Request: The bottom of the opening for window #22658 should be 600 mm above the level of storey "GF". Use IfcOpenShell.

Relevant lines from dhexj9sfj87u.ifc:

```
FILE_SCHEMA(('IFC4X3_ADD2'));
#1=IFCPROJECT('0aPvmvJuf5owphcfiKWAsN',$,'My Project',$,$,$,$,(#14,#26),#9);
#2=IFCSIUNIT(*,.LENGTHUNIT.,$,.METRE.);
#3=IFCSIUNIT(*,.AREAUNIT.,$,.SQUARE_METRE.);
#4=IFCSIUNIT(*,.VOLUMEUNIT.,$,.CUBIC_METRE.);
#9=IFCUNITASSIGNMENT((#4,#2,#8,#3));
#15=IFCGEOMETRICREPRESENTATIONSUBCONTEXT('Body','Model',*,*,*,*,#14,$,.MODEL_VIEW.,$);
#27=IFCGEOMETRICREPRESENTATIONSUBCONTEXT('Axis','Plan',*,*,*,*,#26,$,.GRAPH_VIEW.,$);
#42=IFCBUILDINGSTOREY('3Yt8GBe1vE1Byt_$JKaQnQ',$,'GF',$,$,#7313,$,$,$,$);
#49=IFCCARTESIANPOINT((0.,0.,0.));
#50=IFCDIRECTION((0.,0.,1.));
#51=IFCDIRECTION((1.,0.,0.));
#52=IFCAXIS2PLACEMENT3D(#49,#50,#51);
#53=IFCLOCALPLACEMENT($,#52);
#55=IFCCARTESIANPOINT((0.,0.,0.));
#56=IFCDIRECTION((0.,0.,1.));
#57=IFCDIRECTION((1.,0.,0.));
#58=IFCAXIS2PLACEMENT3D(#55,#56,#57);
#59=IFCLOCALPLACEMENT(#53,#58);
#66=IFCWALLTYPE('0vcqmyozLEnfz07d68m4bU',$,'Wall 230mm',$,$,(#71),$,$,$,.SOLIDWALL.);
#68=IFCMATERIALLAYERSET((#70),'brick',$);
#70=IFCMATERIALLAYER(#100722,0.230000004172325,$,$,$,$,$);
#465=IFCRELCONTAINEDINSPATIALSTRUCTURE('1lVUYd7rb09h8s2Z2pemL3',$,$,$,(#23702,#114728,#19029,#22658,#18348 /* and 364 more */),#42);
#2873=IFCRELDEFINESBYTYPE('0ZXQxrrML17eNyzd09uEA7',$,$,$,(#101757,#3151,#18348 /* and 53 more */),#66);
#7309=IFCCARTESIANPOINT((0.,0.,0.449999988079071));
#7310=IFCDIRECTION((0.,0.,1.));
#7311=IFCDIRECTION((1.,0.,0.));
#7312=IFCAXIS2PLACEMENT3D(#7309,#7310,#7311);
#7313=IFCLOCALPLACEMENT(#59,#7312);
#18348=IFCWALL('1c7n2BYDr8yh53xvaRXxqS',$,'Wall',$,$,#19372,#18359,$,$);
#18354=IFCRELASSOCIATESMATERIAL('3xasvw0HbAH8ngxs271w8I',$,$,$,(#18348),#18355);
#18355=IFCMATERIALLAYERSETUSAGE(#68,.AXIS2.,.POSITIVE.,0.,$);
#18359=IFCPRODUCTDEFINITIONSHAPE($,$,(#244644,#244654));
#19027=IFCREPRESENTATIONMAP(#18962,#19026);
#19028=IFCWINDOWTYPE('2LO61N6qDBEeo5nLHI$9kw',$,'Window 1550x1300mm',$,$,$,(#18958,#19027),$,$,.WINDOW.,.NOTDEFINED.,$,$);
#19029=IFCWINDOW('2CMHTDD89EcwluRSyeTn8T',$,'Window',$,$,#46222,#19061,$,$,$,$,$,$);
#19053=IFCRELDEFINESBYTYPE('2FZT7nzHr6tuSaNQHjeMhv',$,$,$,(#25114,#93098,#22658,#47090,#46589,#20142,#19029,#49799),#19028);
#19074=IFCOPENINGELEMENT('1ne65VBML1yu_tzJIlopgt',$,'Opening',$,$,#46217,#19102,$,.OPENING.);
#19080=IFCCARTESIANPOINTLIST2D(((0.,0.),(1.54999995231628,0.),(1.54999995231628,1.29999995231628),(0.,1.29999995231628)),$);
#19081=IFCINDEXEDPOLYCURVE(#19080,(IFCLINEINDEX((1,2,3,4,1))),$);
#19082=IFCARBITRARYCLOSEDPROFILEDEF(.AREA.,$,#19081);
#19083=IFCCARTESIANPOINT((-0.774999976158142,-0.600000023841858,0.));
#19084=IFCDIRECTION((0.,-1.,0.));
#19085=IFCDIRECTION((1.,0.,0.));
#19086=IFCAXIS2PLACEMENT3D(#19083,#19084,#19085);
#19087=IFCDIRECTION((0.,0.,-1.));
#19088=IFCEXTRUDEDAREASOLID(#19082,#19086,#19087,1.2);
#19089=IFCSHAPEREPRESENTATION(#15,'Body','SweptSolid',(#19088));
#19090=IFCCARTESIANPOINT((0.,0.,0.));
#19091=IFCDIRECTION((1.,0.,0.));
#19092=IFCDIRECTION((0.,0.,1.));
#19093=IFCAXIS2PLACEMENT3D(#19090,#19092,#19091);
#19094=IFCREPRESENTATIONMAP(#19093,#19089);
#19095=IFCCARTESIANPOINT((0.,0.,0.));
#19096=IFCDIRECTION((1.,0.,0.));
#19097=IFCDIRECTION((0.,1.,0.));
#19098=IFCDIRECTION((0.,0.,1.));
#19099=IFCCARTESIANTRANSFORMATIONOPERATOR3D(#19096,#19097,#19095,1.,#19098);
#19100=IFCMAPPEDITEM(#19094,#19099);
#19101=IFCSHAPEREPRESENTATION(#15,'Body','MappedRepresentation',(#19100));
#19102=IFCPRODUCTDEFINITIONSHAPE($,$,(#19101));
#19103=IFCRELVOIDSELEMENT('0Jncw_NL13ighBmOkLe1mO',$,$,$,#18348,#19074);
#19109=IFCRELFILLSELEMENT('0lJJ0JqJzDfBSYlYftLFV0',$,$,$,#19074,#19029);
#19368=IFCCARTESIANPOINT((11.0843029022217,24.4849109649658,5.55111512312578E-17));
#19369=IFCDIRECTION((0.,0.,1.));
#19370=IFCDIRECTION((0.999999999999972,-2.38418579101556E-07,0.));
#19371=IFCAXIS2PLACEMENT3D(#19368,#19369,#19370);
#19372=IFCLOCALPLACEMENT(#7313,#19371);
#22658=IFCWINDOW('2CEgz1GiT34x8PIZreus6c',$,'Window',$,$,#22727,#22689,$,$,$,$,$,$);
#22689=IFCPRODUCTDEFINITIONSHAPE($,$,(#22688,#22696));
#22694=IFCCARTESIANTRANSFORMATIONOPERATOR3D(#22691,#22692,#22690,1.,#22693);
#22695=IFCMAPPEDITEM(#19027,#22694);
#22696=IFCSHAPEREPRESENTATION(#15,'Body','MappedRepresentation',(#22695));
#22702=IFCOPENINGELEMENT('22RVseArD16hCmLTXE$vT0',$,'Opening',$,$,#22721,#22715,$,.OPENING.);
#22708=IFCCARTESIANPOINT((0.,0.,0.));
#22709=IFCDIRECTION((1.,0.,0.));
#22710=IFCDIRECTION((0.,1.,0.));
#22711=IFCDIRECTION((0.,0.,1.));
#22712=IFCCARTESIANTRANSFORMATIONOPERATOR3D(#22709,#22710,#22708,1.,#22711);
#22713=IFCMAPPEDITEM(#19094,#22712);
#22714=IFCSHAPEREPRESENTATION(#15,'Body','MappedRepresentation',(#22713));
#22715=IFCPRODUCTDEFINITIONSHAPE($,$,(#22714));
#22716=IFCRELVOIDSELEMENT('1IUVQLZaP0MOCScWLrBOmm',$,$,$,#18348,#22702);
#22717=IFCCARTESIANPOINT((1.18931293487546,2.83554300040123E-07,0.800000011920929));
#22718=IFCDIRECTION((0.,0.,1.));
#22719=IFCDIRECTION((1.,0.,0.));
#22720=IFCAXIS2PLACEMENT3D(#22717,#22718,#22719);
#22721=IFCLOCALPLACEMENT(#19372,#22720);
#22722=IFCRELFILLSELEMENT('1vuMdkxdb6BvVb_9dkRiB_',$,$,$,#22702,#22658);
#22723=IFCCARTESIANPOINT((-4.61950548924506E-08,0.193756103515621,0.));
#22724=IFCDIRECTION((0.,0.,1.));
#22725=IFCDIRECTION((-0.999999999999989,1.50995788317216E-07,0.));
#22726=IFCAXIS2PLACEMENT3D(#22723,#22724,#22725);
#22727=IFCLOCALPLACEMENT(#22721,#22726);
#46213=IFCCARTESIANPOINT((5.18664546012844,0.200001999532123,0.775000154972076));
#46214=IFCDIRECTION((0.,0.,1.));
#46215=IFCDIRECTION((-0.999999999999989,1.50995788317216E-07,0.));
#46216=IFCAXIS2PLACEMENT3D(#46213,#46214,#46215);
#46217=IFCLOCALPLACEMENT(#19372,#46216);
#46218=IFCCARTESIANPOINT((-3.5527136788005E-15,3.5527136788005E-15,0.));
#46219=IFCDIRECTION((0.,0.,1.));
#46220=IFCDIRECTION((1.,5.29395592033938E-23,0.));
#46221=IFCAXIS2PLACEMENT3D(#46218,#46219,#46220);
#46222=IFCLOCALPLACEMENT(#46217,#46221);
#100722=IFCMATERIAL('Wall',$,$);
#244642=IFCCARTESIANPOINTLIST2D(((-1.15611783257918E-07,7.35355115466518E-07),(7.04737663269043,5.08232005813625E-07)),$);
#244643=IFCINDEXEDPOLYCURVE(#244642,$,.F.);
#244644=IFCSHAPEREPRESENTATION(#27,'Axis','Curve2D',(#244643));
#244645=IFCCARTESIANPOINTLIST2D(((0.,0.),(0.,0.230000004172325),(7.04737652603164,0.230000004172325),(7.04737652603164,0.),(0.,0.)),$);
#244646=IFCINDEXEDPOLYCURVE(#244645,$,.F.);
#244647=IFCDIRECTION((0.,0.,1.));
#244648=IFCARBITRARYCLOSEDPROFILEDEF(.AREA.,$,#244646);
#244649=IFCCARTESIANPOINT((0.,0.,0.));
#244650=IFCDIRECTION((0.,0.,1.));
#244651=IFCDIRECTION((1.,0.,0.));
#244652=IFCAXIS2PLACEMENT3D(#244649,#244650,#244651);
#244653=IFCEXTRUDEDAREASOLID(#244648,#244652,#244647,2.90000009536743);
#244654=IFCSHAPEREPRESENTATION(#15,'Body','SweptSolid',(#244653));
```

```python
import numpy as np
import ifcopenshell
import ifcopenshell.api.geometry
import ifcopenshell.geom
import ifcopenshell.util.element
import ifcopenshell.util.placement
import ifcopenshell.util.shape
import ifcopenshell.util.unit

model = ifcopenshell.open("dhexj9sfj87u.ifc")
unit_scale = ifcopenshell.util.unit.calculate_unit_scale(model)

window = model.by_guid("2CEgz1GiT34x8PIZreus6c")
opening = window.FillsVoids[0].RelatingOpeningElement
storey = ifcopenshell.util.element.get_container(window, ifc_class="IfcBuildingStorey")
level = ifcopenshell.util.placement.get_local_placement(storey.ObjectPlacement)[2, 3]

# The opening's origin need not be at the sill, so measure its lowest point.
shape = ifcopenshell.geom.create_shape(ifcopenshell.geom.settings(), opening)
bottom = ifcopenshell.util.shape.get_shape_bottom_elevation(shape, shape.geometry) / unit_scale
dz = level + 0.6 / unit_scale - bottom

shift = np.array([0.0, 0.0, dz])
# The window is placed relative to its opening, so it follows when the opening moves.
matrix = ifcopenshell.util.placement.get_local_placement(opening.ObjectPlacement)
matrix[:3, 3] += shift
ifcopenshell.api.geometry.edit_object_placement(
    model, product=opening, matrix=matrix, is_si=False, should_transform_children=True
)

print(f"moved by {dz * unit_scale:+.3f} m")

model.write("dhexj9sfj87u_v2.ifc")
```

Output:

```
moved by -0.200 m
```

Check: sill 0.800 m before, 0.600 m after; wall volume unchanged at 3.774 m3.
